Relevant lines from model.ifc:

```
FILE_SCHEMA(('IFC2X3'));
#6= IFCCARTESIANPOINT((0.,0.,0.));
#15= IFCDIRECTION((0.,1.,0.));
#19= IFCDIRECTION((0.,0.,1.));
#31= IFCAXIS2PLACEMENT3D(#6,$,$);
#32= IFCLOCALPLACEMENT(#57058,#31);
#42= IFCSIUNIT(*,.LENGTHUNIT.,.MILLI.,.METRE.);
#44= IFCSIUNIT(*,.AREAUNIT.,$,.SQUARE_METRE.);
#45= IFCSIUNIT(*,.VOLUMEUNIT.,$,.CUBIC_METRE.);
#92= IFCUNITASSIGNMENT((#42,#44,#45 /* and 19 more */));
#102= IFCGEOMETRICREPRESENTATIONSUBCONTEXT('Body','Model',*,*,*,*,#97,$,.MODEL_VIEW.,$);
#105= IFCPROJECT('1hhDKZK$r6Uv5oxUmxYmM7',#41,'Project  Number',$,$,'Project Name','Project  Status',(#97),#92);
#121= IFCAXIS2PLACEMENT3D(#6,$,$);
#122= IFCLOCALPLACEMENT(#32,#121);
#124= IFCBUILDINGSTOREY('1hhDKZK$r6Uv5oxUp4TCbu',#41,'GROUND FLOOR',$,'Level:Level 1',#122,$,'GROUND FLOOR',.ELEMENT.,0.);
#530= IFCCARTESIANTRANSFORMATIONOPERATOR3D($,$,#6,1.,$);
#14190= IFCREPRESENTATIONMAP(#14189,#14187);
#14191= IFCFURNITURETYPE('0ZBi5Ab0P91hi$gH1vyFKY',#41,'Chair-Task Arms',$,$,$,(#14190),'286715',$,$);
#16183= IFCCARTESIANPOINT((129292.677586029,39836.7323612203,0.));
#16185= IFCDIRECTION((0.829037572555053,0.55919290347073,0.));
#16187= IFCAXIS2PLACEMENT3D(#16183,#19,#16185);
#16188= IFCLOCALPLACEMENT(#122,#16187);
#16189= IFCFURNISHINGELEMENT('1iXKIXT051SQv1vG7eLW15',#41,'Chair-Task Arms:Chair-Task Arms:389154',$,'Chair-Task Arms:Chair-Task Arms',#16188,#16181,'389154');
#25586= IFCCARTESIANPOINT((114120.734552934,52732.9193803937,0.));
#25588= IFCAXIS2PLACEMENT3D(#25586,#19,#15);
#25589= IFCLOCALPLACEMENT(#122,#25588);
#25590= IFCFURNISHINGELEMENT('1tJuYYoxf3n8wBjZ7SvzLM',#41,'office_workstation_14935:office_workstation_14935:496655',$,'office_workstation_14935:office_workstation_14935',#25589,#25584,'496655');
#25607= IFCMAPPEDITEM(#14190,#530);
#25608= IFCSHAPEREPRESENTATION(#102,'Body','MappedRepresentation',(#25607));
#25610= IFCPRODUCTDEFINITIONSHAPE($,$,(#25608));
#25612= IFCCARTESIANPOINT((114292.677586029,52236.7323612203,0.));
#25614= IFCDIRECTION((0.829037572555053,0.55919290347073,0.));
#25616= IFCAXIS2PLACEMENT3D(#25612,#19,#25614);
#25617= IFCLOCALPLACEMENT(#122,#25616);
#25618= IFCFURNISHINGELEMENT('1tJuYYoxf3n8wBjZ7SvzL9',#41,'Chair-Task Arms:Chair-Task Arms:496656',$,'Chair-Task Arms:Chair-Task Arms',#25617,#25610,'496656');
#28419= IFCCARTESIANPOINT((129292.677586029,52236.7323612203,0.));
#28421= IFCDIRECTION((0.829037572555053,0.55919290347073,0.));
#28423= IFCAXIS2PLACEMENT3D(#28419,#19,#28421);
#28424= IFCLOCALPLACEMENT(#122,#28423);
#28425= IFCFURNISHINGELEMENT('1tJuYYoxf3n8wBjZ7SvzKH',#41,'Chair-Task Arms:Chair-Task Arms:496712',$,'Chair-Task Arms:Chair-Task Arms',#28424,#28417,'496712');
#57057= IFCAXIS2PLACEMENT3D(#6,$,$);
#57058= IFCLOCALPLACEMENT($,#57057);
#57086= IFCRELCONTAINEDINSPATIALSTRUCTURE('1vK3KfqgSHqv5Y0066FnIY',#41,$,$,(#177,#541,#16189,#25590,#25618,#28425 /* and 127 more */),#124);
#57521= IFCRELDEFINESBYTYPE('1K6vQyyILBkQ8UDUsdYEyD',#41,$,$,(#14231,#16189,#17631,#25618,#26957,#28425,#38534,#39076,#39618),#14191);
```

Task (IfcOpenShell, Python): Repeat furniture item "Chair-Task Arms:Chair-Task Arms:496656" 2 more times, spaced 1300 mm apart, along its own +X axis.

```python
import ifcopenshell
import ifcopenshell.api.geometry
import ifcopenshell.api.root
import ifcopenshell.util.element
import ifcopenshell.util.placement
import ifcopenshell.util.unit

model = ifcopenshell.open("model.ifc")
unit_scale = ifcopenshell.util.unit.calculate_unit_scale(model)


def reuse_history(source, copy):
    """copy_class also copies each property set's owner history, people and application; keep the originals."""
    for rel in copy.IsDefinedBy:
        if rel.is_a("IfcRelDefinesByProperties") and (history := rel.RelatingPropertyDefinition.OwnerHistory):
            rel.RelatingPropertyDefinition.OwnerHistory = source.OwnerHistory
            ifcopenshell.util.element.remove_deep2(model, history)


source = model.by_guid("1tJuYYoxf3n8wBjZ7SvzL9")
base = ifcopenshell.util.placement.get_local_placement(source.ObjectPlacement)
step = base[:3, 0] * 1.3 / unit_scale

for i in range(1, 3):
    copy = ifcopenshell.api.root.copy_class(model, product=source)
    copy.Representation = ifcopenshell.util.element.copy_deep(
        model, source.Representation, exclude=["IfcGeometricRepresentationContext", "IfcRepresentationMap"]
    )
    copy.Name = "Chair-Task Arms:Chair-Task Arms"
    copy.Tag = None
    reuse_history(source, copy)
    matrix = base.copy()
    matrix[:3, 3] += i * step
    print("added at", matrix[:3, 3].round(3) + 0.0)
    ifcopenshell.api.geometry.edit_object_placement(model, product=copy, matrix=matrix, is_si=False)

model.write("model_updated.ifc")
```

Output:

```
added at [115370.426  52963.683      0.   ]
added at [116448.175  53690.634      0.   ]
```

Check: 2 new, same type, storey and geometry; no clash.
